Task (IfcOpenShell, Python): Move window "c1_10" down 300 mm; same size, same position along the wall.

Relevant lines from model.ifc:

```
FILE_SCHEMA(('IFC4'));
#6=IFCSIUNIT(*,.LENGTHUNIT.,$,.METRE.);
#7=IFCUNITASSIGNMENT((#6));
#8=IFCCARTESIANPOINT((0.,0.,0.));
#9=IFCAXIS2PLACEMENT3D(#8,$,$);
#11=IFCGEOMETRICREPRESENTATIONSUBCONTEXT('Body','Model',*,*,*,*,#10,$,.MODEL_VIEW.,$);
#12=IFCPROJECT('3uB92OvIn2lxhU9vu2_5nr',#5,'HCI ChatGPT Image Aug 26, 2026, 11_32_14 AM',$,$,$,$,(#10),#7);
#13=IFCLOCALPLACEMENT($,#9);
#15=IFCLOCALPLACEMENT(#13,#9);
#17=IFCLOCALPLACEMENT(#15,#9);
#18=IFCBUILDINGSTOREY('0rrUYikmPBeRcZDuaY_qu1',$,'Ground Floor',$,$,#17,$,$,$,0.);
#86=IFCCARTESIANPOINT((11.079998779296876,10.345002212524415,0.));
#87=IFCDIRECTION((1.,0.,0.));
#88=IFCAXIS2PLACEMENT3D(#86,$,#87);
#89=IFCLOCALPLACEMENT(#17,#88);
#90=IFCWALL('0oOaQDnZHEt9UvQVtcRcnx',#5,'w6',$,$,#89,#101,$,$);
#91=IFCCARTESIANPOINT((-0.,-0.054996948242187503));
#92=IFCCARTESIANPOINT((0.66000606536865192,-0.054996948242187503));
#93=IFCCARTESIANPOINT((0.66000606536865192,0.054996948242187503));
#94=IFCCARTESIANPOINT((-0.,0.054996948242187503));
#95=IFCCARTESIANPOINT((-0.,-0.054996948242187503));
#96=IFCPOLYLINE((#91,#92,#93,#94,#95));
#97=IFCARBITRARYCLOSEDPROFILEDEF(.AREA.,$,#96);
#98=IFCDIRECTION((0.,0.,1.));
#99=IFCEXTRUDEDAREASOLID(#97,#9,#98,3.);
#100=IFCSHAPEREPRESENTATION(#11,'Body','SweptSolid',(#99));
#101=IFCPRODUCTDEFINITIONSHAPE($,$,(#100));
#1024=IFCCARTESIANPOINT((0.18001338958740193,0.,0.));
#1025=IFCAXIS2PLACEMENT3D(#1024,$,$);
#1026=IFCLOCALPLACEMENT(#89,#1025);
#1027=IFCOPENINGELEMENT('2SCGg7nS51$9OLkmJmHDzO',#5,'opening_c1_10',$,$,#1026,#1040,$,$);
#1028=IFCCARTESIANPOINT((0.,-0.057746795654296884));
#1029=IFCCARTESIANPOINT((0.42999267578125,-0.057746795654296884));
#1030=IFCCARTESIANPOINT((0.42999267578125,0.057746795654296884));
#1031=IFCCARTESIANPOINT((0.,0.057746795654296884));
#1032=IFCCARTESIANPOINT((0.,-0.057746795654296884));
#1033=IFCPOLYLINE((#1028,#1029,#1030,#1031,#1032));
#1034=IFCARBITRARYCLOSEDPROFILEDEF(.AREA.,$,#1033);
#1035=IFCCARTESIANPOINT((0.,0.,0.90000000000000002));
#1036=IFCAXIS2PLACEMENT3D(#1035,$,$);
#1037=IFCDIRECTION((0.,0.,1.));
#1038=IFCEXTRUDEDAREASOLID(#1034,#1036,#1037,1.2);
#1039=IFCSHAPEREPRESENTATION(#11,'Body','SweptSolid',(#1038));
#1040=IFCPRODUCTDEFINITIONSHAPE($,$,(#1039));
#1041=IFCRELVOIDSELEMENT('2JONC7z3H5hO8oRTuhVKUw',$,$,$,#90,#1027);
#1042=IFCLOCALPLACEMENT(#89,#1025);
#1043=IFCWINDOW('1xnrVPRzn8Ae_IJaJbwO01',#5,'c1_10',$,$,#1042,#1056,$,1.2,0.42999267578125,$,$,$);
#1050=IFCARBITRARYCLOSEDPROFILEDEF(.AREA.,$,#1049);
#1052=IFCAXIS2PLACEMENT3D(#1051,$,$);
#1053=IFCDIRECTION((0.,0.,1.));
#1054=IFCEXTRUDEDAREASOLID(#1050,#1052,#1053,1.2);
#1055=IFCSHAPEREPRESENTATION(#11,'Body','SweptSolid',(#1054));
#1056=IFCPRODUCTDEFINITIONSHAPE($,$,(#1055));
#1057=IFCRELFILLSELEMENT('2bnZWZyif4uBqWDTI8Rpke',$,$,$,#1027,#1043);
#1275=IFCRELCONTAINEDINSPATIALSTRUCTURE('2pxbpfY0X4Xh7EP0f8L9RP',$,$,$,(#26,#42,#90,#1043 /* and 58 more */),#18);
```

```python
import numpy as np
import ifcopenshell
import ifcopenshell.api.geometry
import ifcopenshell.util.placement
import ifcopenshell.util.unit

model = ifcopenshell.open("model.ifc")
unit_scale = ifcopenshell.util.unit.calculate_unit_scale(model)

window = model.by_guid("1xnrVPRzn8Ae_IJaJbwO01")
opening = window.FillsVoids[0].RelatingOpeningElement
dz = -0.3 / unit_scale

shift = np.array([0.0, 0.0, dz])
# The window is not placed relative to its opening, so move both.
for product in (opening, window):
    matrix = ifcopenshell.util.placement.get_local_placement(product.ObjectPlacement)
    matrix[:3, 3] += shift
    ifcopenshell.api.geometry.edit_object_placement(model, product=product, matrix=matrix, is_si=False)

print(f"moved by {dz * unit_scale:+.3f} m")

model.write("model_edited.ifc")
```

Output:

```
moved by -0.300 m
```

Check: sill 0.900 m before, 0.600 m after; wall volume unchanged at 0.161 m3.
